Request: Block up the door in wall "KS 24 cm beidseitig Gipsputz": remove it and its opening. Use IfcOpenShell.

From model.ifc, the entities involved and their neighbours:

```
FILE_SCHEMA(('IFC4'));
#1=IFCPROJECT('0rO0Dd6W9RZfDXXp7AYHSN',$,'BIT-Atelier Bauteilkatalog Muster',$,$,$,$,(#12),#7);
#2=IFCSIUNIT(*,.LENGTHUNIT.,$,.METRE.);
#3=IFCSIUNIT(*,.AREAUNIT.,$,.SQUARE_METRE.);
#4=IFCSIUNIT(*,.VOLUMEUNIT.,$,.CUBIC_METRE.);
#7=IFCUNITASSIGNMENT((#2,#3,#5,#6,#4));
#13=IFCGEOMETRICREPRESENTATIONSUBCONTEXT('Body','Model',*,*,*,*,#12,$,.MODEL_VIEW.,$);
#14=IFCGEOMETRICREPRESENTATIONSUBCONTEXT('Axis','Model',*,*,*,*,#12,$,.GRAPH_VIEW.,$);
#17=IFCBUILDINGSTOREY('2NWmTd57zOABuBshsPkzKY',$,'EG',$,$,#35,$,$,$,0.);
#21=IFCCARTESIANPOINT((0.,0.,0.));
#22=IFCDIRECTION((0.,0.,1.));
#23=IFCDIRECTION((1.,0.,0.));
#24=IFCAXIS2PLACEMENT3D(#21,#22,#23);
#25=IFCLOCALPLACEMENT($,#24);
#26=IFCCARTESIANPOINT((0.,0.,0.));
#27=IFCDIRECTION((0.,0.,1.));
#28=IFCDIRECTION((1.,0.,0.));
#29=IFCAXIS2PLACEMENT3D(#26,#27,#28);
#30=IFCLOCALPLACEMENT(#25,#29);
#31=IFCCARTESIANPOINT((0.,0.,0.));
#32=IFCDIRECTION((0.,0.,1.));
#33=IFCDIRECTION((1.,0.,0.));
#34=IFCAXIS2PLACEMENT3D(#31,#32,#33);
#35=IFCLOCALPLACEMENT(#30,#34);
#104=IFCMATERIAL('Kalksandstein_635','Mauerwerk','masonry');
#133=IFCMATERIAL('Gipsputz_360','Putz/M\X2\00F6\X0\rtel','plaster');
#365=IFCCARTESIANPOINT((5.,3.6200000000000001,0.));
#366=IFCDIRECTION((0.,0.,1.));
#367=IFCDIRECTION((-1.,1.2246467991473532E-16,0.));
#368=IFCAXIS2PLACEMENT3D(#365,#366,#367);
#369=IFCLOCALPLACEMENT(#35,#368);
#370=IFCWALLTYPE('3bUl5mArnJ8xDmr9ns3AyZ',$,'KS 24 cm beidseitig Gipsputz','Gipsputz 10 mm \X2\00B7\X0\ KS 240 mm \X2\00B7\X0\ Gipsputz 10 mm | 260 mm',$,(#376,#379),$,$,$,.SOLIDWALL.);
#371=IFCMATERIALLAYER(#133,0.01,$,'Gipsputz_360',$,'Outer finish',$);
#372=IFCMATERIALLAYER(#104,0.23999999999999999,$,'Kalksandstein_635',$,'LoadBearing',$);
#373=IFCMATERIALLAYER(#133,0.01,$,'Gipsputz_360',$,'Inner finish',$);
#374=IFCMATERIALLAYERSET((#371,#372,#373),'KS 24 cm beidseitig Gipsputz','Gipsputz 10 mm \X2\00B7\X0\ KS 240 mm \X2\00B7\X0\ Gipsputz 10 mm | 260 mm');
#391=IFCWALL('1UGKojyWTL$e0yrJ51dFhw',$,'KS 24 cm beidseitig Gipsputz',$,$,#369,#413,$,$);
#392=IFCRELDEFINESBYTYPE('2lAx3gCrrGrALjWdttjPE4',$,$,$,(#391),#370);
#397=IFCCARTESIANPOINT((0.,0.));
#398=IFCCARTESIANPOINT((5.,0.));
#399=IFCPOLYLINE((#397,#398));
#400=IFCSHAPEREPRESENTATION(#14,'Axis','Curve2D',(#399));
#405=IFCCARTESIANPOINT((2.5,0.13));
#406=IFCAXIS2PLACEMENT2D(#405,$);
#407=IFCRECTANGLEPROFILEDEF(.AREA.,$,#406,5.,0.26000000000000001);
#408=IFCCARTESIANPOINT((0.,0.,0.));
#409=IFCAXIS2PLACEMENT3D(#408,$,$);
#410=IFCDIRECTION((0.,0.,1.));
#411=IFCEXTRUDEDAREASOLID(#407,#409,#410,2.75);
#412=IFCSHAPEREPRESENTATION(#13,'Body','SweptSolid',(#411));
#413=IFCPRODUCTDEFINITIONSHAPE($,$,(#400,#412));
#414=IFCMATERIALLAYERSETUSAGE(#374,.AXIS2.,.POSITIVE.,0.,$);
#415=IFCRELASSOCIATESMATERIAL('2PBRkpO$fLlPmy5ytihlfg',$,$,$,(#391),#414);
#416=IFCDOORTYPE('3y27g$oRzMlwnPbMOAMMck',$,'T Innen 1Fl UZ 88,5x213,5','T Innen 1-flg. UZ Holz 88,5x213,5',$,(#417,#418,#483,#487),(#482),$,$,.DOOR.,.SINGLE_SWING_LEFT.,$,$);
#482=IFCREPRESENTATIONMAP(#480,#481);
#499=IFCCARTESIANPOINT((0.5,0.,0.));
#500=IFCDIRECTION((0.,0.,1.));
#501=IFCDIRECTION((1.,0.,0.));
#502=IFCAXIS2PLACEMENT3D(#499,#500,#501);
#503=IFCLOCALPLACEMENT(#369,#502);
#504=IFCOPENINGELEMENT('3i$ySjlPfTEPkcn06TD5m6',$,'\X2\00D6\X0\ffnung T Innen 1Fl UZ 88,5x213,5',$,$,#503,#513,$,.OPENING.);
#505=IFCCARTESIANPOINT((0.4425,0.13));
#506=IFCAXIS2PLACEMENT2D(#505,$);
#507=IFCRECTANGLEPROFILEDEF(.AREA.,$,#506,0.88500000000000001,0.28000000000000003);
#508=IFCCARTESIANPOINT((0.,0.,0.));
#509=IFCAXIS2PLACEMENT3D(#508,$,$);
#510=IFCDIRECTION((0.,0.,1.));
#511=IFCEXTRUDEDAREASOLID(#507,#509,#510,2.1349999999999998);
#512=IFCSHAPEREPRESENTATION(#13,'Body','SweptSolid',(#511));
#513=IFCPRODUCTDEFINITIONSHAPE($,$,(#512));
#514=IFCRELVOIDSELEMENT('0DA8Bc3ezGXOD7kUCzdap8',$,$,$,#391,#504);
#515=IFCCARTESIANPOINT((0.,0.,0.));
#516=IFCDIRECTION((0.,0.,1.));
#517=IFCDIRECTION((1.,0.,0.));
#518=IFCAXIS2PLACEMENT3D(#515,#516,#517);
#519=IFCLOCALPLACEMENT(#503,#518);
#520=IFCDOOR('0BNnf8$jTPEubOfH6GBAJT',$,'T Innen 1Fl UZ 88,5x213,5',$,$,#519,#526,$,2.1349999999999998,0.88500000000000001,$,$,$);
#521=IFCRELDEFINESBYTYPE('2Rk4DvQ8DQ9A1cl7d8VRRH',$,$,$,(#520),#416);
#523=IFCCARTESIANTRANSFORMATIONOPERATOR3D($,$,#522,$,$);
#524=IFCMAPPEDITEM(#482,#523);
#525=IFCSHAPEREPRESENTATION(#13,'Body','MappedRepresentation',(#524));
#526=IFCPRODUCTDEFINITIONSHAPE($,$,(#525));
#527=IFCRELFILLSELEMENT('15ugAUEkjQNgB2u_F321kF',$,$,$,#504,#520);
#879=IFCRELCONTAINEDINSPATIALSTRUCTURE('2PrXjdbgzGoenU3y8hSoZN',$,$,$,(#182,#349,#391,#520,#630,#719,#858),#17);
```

```python
import ifcopenshell
import ifcopenshell.api.feature
import ifcopenshell.api.root
import ifcopenshell.geom
import ifcopenshell.util.shape

model = ifcopenshell.open("model.ifc")
settings = ifcopenshell.geom.settings()


def volume(element):
    """Net volume in cubic metres, openings subtracted."""
    shape = ifcopenshell.geom.create_shape(settings, element)
    return ifcopenshell.util.shape.get_volume(shape.geometry)


door = model.by_guid("0BNnf8$jTPEubOfH6GBAJT")
opening = door.FillsVoids[0].RelatingOpeningElement
wall = opening.VoidsElements[0].RelatingBuildingElement
before = volume(wall)

ifcopenshell.api.root.remove_product(model, product=door)
ifcopenshell.api.feature.remove_feature(model, feature=opening)

after = volume(wall)

print(f"wall volume {before:.3f} -> {after:.3f} m3")

model.write("model-out.ifc")
```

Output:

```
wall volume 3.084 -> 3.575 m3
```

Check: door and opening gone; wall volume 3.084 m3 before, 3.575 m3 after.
